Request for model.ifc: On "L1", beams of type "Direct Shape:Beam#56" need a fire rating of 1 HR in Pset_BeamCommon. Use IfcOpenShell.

First a look at what the model holds.

```python
import ifcopenshell
import ifcopenshell.util.element

model = ifcopenshell.open("model.ifc")
print(model.schema)
storey = next(s for s in model.by_type("IfcBuildingStorey") if s.Name == "L1")
beams = [e for e in ifcopenshell.util.element.get_decomposition(storey) if e.is_a("IfcBeam")]
seen = {}
for e in beams:
    element_type = ifcopenshell.util.element.get_type(e)
    key = (element_type.Name if element_type != e and element_type else None, ifcopenshell.util.element.get_pset(e, "Pset_BeamCommon", "FireRating"))
    seen[key] = seen.get(key, 0) + 1
for (name, value), count in sorted(seen.items(), key=str):
    print(count, "x", name, "|", value)
```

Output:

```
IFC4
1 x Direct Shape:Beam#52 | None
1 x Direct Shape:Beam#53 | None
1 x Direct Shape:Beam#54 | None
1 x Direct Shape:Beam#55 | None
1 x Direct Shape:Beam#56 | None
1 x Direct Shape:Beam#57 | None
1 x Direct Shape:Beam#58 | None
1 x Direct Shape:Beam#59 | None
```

```python
import ifcopenshell
import ifcopenshell.api.pset
import ifcopenshell.util.element

model = ifcopenshell.open("model.ifc")

storey = next(s for s in model.by_type("IfcBuildingStorey") if s.Name == "L1")
beams = [e for e in ifcopenshell.util.element.get_decomposition(storey) if e.is_a("IfcBeam")]

count = 0
for e in beams:
    element_type = ifcopenshell.util.element.get_type(e)
    if element_type in (None, e) or element_type.Name != "Direct Shape:Beam#56":
        continue
    # add_pset returns the element's existing set when there is one.
    pset = ifcopenshell.api.pset.add_pset(model, product=e, name="Pset_BeamCommon")
    ifcopenshell.api.pset.edit_pset(model, pset=pset, properties={"FireRating": "1 HR"})
    count += 1

print(count, "beams updated")

model.write("model-out.ifc")
```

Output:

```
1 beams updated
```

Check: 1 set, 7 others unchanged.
